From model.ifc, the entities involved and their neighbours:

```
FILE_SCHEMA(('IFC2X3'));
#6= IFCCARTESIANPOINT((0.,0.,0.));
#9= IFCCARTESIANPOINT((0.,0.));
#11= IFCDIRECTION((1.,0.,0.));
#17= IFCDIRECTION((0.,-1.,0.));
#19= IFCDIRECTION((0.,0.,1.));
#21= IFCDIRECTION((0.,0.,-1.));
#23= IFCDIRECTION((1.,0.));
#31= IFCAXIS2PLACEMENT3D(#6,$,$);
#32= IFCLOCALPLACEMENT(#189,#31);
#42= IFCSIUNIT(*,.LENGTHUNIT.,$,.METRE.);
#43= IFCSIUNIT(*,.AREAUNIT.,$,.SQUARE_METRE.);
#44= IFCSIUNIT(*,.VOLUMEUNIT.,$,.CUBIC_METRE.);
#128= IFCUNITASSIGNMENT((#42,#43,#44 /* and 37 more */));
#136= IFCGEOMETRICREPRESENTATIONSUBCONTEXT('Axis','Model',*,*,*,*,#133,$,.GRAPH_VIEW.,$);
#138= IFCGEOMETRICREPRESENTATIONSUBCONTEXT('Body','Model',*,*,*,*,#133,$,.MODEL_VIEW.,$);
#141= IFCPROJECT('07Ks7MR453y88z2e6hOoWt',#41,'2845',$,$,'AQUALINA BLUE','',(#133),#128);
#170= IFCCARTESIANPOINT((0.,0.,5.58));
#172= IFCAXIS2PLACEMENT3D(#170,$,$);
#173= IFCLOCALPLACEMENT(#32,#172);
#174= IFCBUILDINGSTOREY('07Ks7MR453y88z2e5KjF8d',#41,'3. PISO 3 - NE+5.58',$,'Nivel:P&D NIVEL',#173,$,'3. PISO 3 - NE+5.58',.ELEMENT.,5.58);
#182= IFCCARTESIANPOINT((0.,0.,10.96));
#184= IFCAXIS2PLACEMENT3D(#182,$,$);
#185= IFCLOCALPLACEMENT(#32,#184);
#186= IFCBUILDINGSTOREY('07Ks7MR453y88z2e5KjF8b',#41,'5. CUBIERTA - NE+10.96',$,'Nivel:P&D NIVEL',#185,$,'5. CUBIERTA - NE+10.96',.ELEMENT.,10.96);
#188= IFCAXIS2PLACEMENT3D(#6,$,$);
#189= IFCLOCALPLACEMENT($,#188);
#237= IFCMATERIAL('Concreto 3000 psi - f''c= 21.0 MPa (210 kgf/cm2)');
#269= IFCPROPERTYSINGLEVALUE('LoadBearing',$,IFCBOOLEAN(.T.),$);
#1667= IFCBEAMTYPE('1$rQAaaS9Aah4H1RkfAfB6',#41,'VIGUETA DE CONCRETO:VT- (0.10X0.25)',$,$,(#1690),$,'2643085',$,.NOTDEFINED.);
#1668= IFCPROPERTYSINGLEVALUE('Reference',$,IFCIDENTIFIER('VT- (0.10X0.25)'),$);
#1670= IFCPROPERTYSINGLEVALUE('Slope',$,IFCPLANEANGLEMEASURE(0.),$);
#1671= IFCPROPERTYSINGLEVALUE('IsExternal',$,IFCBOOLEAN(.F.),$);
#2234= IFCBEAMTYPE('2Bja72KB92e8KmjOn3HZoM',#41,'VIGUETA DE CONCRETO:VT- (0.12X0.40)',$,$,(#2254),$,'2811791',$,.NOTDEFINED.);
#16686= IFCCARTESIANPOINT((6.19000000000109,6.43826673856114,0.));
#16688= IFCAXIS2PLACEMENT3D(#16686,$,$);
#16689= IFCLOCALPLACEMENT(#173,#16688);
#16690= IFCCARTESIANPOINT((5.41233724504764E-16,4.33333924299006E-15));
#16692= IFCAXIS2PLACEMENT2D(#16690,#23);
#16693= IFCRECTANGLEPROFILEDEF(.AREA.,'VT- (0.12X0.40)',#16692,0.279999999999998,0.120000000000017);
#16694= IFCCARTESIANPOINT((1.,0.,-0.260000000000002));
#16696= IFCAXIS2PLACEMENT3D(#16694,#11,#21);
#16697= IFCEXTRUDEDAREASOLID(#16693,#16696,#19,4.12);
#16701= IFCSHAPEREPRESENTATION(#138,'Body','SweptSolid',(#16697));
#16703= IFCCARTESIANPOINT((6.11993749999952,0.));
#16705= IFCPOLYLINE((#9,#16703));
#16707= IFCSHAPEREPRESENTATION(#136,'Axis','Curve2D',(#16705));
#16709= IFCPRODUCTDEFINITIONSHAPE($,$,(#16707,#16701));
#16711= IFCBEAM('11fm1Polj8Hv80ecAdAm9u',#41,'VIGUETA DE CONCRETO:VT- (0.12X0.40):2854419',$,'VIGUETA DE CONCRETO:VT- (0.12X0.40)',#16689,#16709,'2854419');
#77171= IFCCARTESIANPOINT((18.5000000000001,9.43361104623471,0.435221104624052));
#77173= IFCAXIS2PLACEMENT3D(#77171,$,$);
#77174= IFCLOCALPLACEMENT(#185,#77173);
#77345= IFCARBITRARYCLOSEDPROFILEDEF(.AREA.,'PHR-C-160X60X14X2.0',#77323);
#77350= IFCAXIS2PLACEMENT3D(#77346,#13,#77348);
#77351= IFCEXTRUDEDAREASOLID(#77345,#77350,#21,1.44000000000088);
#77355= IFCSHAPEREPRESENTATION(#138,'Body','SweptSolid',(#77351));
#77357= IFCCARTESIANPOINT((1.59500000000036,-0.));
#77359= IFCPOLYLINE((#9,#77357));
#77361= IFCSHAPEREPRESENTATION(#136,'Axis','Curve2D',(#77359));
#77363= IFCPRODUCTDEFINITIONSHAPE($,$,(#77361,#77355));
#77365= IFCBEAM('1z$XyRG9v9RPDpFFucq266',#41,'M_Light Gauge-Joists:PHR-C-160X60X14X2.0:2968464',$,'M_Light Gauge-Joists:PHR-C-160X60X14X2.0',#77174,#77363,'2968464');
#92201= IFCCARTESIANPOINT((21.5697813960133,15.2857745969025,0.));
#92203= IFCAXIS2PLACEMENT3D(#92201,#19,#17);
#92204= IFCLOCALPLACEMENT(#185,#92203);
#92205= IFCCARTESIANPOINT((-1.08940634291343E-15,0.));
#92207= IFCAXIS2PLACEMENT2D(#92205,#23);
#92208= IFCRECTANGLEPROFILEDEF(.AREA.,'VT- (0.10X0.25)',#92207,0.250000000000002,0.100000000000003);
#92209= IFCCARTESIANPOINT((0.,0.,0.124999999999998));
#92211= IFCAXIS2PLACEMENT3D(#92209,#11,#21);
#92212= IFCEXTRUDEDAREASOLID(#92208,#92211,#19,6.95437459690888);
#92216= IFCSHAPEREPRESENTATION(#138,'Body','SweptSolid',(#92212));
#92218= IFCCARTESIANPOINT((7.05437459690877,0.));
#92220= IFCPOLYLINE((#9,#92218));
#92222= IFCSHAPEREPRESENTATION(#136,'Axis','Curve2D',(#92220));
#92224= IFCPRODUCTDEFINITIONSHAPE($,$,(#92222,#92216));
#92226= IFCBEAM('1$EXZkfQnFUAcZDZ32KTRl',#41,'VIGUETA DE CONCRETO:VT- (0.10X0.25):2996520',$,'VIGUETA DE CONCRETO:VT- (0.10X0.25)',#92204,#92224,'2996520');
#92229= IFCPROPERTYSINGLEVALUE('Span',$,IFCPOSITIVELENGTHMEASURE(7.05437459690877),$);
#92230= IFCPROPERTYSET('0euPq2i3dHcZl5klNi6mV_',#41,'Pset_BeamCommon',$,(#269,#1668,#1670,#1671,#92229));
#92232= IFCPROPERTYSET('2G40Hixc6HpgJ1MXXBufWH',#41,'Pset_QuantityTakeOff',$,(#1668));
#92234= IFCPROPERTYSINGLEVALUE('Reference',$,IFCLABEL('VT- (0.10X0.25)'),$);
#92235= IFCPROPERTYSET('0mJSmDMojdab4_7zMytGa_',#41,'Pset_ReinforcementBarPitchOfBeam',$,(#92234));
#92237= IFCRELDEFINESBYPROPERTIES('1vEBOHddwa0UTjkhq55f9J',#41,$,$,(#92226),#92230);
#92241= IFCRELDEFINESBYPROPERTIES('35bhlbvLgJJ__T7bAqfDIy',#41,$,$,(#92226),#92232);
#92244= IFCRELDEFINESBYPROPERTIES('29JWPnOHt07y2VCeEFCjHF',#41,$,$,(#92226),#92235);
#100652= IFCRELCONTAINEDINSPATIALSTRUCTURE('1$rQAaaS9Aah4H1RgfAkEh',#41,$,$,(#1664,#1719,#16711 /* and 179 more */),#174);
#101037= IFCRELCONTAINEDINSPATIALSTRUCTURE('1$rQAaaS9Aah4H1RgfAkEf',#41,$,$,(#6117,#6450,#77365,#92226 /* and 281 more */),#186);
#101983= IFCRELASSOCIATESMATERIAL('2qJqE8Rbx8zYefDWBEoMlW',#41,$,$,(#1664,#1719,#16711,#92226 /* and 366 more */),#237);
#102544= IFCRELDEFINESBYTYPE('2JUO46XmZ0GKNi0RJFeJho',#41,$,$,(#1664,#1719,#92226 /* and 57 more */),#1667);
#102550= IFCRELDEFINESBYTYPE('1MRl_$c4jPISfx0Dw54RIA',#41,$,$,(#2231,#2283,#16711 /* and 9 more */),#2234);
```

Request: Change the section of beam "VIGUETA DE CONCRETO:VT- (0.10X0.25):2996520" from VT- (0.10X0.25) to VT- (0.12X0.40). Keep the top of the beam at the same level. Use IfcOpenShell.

```python
import ifcopenshell
import ifcopenshell.api.pset
import ifcopenshell.api.type
import ifcopenshell.util.element
import ifcopenshell.util.representation

model = ifcopenshell.open("model.ifc")

member = model.by_guid("1$EXZkfQnFUAcZDZ32KTRl")
source = next(p for p in model.by_type("IfcRectangleProfileDef") if p.ProfileName == "VT- (0.12X0.40)")

body = ifcopenshell.util.representation.get_representation(member, "Model", "Body")
solid = body.Items[0]
old_profile = solid.SweptArea

# Copy the section's sizes but keep this member's own profile position.
profile = ifcopenshell.util.element.copy(model, source)
# Profiles are centred, so shift by half the change in depth to hold the top.
shift = (old_profile.XDim - profile.XDim) / 2
x, y = old_profile.Position.Location.Coordinates
up = (-1.0, 0.0)  # upwards, in the solid's own plane
location = model.createIfcCartesianPoint((x + up[0] * shift, y + up[1] * shift))
profile.Position = model.createIfcAxis2Placement2D(location, old_profile.Position.RefDirection)
solid.SweptArea = profile
if not model.get_total_inverses(old_profile):
    ifcopenshell.util.element.remove_deep2(model, old_profile)

new_type = model.by_id(2234)
ifcopenshell.api.type.assign_type(
    model, related_objects=[member], relating_type=new_type, should_map_representations=False
)
member.Name = member.Name.replace("VT- (0.10X0.25)", "VT- (0.12X0.40)")
member.ObjectType = "VIGUETA DE CONCRETO:VT- (0.12X0.40)"
pset = model.by_id(ifcopenshell.util.element.get_pset(member, "Pset_BeamCommon", should_inherit=False)["id"])
ifcopenshell.api.pset.edit_pset(model, pset=pset, properties={"Reference": "VT- (0.12X0.40)"})
pset = model.by_id(ifcopenshell.util.element.get_pset(member, "Pset_QuantityTakeOff", should_inherit=False)["id"])
ifcopenshell.api.pset.edit_pset(model, pset=pset, properties={"Reference": "VT- (0.12X0.40)"})
pset = model.by_id(ifcopenshell.util.element.get_pset(member, "Pset_ReinforcementBarPitchOfBeam", should_inherit=False)["id"])
ifcopenshell.api.pset.edit_pset(model, pset=pset, properties={"Reference": "VT- (0.12X0.40)"})

print(solid.SweptArea)

model.write("model_edited.ifc")
```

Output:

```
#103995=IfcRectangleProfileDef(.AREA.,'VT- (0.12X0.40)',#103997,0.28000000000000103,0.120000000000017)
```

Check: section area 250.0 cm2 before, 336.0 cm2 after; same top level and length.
